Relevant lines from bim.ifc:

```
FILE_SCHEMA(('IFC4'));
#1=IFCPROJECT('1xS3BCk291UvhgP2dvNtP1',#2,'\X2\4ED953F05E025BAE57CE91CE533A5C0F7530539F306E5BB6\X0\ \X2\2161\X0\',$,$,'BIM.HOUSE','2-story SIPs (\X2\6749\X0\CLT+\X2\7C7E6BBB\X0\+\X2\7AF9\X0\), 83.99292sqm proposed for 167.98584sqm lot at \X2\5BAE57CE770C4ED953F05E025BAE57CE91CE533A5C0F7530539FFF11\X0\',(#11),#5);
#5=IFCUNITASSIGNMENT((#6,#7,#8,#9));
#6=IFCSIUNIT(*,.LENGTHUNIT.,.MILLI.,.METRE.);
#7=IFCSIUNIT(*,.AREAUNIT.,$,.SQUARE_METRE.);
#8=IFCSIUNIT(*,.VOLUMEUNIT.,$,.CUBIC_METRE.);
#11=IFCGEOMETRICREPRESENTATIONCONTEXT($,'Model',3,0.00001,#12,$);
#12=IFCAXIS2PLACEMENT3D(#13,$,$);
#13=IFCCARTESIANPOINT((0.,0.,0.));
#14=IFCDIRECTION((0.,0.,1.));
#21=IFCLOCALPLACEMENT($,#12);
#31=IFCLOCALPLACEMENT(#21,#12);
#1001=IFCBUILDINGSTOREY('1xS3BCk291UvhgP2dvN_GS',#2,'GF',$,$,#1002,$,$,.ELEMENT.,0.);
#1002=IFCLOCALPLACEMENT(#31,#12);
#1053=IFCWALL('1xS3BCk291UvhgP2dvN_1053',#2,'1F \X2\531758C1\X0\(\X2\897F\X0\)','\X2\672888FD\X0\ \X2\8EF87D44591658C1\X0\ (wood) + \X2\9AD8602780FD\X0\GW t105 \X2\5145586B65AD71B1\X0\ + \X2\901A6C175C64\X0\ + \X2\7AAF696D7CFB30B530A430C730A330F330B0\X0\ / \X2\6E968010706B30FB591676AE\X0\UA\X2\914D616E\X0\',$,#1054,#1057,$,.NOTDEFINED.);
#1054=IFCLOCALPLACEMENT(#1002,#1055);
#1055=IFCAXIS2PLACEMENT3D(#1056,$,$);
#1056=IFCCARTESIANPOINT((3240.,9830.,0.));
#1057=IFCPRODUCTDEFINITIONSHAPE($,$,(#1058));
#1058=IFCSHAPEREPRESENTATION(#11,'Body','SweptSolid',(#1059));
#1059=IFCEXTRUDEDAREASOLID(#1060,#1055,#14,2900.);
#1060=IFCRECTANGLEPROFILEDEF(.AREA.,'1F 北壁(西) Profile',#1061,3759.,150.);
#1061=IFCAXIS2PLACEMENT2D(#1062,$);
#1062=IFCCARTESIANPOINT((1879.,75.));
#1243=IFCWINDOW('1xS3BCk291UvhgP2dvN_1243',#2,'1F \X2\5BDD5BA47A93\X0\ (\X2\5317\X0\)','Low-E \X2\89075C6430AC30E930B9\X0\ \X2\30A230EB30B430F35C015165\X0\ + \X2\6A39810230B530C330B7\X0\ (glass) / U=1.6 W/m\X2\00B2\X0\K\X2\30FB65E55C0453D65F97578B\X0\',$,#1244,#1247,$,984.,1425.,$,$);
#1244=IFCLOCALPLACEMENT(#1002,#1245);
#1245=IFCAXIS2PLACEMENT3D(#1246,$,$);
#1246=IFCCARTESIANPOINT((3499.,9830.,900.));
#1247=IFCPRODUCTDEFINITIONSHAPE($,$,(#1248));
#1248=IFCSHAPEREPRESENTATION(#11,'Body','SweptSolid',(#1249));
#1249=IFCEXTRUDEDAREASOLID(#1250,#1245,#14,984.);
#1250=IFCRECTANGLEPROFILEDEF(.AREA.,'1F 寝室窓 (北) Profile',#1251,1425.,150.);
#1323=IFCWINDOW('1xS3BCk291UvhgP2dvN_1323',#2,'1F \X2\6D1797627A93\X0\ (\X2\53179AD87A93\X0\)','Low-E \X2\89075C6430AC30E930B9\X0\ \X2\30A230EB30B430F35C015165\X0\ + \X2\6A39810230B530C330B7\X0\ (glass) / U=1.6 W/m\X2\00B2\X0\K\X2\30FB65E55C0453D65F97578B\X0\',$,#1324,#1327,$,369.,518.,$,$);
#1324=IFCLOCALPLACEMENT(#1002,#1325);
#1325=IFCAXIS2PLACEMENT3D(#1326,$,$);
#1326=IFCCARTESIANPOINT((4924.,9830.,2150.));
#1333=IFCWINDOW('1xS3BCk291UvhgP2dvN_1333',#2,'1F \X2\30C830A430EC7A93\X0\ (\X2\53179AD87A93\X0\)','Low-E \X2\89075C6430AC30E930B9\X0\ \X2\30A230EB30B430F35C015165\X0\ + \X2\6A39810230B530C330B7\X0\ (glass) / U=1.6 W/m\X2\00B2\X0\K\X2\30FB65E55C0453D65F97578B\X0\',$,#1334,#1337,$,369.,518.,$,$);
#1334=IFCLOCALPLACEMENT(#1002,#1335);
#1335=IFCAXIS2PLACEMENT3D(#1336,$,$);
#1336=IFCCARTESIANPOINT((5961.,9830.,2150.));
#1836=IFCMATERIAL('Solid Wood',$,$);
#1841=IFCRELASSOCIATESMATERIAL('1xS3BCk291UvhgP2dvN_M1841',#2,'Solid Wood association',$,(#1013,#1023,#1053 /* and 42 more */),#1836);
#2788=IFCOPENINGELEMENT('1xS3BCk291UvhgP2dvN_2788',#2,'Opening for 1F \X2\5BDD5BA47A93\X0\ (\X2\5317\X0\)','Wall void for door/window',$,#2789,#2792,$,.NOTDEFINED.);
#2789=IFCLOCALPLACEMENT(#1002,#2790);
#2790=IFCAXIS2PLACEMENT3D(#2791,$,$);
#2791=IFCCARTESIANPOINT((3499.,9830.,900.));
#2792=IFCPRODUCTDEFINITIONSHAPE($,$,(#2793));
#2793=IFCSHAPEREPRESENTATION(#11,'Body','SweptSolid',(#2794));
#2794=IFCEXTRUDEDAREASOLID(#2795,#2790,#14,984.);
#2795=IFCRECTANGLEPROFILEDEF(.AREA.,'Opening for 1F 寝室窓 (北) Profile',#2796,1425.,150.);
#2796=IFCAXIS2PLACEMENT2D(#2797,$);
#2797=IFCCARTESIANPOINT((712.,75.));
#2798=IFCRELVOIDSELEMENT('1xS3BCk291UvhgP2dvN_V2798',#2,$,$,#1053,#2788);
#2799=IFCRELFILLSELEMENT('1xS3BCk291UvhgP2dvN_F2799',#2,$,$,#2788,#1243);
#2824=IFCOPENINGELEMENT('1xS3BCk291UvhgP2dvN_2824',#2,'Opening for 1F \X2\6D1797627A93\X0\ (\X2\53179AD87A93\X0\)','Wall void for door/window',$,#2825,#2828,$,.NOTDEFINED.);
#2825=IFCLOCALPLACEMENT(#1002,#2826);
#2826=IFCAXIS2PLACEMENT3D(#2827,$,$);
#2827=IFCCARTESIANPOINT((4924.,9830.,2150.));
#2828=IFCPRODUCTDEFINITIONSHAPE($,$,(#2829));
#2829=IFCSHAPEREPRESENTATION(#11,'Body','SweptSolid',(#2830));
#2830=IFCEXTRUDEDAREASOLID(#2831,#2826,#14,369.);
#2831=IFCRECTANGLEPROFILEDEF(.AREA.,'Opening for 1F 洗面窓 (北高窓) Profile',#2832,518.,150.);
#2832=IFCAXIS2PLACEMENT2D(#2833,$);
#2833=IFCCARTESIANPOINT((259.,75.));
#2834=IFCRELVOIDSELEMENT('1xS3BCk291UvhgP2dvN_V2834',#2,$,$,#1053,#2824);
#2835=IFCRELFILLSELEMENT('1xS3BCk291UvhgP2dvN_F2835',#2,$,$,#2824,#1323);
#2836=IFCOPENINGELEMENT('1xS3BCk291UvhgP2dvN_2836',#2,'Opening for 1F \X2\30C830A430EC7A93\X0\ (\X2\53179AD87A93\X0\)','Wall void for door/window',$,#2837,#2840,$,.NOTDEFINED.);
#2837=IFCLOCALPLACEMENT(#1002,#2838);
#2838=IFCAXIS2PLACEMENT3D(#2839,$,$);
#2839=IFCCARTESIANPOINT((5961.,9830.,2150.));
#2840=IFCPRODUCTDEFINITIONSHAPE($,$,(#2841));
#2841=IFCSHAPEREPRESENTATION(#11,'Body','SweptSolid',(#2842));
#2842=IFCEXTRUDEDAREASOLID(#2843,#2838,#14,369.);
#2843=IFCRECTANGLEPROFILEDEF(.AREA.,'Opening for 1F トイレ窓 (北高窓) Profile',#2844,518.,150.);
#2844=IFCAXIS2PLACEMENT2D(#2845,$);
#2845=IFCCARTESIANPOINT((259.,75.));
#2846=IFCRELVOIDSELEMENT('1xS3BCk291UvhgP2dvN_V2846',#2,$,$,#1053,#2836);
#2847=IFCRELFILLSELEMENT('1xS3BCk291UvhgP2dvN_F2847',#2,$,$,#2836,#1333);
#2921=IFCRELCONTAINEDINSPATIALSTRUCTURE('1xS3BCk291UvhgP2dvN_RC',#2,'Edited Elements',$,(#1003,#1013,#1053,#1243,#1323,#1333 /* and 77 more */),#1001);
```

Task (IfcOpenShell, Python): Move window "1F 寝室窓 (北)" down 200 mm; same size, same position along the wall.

```python
import numpy as np
import ifcopenshell
import ifcopenshell.api.geometry
import ifcopenshell.util.placement
import ifcopenshell.util.unit

model = ifcopenshell.open("bim.ifc")
unit_scale = ifcopenshell.util.unit.calculate_unit_scale(model)

window = model.by_guid("1xS3BCk291UvhgP2dvN_1243")
opening = window.FillsVoids[0].RelatingOpeningElement
dz = -0.2 / unit_scale

shift = np.array([0.0, 0.0, dz])
# The window is not placed relative to its opening, so move both.
for product in (opening, window):
    matrix = ifcopenshell.util.placement.get_local_placement(product.ObjectPlacement)
    matrix[:3, 3] += shift
    ifcopenshell.api.geometry.edit_object_placement(model, product=product, matrix=matrix, is_si=False)

print(f"moved by {dz * unit_scale:+.3f} m")

model.write("bim_v2.ifc")
```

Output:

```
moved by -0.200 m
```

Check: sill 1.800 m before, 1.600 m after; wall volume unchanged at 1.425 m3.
